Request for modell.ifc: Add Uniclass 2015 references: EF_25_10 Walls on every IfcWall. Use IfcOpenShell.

First a look at what the model holds.

```python
import ifcopenshell

model = ifcopenshell.open("modell.ifc")
print(model.schema)
print("classifications:", [c.Name for c in model.by_type("IfcClassification")])
for ifc_class in ("IfcDoor", "IfcRoof", "IfcStair", "IfcWall", "IfcWindow"):
    print(ifc_class, len(model.by_type(ifc_class)))
```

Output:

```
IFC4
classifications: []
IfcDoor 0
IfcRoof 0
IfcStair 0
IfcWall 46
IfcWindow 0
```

```python
import ifcopenshell
import ifcopenshell.api.classification

model = ifcopenshell.open("modell.ifc")

system = ifcopenshell.api.classification.add_classification(model, classification="Uniclass 2015")

codes = {
    "IfcWall": ("EF_25_10", "Walls"),
}
for ifc_class, (code, name) in codes.items():
    products = model.by_type(ifc_class)
    ifcopenshell.api.classification.add_reference(
        model, products=products, classification=system, identification=code, name=name
    )
    print(code, len(products))

model.write("modell_edited.ifc")
```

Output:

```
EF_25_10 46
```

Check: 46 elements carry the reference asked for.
